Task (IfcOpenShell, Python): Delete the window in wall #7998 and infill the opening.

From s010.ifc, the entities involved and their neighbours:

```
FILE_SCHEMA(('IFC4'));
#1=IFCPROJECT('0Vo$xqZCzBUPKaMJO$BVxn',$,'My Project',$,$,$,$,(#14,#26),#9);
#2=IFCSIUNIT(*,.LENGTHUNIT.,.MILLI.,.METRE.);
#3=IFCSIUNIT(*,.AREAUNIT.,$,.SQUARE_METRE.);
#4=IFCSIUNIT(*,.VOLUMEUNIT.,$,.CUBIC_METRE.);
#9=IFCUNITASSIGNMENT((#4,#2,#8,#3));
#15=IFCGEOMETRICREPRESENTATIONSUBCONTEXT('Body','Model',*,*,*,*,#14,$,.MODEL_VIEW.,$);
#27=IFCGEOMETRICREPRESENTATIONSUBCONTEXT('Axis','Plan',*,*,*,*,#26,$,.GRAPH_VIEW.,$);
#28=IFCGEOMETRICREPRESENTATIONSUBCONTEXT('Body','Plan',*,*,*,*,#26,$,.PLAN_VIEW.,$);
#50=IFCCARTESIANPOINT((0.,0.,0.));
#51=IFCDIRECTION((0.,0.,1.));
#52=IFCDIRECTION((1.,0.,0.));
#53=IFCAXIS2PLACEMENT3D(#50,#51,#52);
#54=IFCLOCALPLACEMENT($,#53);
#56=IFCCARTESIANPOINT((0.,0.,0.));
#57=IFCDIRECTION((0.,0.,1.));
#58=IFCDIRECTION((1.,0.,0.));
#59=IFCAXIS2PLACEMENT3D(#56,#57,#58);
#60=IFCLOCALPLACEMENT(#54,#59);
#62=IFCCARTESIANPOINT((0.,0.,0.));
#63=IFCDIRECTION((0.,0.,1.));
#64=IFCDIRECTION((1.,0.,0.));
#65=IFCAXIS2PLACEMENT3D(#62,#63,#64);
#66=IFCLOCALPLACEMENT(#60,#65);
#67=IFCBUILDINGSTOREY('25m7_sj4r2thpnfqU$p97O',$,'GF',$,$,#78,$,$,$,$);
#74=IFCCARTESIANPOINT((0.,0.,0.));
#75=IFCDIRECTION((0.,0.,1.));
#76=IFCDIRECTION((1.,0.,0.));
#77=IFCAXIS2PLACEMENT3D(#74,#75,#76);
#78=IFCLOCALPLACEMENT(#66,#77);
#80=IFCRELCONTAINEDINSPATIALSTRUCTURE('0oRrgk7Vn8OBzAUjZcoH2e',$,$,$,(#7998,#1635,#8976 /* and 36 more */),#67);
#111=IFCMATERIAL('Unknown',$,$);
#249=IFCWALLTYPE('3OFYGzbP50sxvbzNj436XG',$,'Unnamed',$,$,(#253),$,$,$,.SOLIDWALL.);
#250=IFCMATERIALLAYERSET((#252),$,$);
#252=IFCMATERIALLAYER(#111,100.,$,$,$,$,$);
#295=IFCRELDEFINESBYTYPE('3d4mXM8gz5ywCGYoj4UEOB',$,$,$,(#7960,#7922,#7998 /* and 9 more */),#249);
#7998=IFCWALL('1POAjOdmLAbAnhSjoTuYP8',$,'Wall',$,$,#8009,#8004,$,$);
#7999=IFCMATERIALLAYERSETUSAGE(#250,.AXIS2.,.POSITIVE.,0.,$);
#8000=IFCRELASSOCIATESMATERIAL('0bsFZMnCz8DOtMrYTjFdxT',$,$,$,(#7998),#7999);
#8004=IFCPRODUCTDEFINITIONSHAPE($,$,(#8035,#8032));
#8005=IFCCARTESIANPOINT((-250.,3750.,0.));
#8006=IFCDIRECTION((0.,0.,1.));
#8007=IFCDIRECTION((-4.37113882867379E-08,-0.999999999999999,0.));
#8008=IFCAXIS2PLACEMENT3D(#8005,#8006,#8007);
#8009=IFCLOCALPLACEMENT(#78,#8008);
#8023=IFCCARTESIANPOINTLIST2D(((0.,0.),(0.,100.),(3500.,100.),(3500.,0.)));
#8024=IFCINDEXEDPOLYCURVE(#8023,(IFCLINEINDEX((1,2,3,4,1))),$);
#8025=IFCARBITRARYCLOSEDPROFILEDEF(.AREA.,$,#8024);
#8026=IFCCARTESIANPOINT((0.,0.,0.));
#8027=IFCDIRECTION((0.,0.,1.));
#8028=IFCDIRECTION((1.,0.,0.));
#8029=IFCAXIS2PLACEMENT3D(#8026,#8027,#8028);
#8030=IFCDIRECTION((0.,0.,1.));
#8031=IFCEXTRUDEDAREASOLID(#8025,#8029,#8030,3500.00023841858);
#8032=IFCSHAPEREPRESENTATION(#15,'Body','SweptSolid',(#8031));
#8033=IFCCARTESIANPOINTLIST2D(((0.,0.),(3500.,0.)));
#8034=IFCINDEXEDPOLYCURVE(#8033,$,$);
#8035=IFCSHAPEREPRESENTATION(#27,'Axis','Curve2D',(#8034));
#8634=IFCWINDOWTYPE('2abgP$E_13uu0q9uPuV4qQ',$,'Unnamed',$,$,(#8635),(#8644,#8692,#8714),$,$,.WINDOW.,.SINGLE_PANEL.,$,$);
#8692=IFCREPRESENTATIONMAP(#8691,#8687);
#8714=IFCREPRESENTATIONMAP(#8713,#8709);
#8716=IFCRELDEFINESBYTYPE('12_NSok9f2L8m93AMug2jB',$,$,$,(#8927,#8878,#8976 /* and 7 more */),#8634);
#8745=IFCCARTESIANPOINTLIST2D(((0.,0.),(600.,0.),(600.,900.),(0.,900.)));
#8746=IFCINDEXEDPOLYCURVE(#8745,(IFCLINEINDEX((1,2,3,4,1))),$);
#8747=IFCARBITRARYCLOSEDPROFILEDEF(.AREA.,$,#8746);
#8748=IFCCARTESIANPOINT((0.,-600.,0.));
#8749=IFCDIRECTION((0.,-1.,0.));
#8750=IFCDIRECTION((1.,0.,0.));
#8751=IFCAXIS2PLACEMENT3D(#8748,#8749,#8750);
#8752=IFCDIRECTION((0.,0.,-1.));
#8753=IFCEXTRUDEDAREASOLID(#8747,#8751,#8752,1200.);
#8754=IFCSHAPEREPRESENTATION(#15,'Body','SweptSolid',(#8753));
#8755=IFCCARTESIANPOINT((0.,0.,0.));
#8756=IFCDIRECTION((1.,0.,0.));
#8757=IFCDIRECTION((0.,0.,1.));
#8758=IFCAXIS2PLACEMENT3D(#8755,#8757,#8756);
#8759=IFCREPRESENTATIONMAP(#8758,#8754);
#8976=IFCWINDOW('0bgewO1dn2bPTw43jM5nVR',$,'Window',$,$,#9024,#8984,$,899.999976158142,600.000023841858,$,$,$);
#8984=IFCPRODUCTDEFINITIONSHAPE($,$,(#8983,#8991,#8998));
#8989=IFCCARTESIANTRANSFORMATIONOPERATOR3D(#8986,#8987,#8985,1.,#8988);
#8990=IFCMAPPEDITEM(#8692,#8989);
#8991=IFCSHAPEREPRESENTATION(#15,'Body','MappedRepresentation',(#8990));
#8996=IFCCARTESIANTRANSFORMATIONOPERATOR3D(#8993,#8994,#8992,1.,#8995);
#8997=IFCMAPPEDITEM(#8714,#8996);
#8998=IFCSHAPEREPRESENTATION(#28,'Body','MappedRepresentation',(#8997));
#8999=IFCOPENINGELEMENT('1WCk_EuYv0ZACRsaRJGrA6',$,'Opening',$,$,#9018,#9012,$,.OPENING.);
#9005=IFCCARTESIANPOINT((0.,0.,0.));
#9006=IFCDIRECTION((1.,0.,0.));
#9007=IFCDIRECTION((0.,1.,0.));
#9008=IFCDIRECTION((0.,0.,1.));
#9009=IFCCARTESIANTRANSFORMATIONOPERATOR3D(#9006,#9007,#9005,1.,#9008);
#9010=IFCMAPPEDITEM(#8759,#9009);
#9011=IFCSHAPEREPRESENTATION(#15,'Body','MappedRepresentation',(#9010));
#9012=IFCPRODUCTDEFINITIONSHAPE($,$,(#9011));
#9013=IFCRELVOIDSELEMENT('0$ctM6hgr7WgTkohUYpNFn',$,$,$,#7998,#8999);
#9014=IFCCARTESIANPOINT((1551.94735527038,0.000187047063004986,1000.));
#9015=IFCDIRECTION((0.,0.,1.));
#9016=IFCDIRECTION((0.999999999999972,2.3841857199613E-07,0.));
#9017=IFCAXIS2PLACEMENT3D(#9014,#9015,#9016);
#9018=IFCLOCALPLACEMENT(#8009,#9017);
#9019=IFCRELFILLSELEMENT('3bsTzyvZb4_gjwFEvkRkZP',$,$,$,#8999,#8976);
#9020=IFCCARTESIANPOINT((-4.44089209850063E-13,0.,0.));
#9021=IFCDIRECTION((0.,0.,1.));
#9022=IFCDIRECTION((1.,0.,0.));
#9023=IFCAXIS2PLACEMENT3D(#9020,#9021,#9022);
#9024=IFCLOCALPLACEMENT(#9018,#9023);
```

```python
import ifcopenshell
import ifcopenshell.api.feature
import ifcopenshell.api.root
import ifcopenshell.geom
import ifcopenshell.util.shape

model = ifcopenshell.open("s010.ifc")
settings = ifcopenshell.geom.settings()


def volume(element):
    """Net volume in cubic metres, openings subtracted."""
    shape = ifcopenshell.geom.create_shape(settings, element)
    return ifcopenshell.util.shape.get_volume(shape.geometry)


window = model.by_id(8976)
opening = window.FillsVoids[0].RelatingOpeningElement
wall = opening.VoidsElements[0].RelatingBuildingElement
before = volume(wall)

ifcopenshell.api.root.remove_product(model, product=window)
ifcopenshell.api.feature.remove_feature(model, feature=opening)

after = volume(wall)

print(f"wall volume {before:.3f} -> {after:.3f} m3")

model.write("s010_updated.ifc")
```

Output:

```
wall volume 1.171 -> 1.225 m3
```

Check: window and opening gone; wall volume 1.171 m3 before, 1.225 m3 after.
